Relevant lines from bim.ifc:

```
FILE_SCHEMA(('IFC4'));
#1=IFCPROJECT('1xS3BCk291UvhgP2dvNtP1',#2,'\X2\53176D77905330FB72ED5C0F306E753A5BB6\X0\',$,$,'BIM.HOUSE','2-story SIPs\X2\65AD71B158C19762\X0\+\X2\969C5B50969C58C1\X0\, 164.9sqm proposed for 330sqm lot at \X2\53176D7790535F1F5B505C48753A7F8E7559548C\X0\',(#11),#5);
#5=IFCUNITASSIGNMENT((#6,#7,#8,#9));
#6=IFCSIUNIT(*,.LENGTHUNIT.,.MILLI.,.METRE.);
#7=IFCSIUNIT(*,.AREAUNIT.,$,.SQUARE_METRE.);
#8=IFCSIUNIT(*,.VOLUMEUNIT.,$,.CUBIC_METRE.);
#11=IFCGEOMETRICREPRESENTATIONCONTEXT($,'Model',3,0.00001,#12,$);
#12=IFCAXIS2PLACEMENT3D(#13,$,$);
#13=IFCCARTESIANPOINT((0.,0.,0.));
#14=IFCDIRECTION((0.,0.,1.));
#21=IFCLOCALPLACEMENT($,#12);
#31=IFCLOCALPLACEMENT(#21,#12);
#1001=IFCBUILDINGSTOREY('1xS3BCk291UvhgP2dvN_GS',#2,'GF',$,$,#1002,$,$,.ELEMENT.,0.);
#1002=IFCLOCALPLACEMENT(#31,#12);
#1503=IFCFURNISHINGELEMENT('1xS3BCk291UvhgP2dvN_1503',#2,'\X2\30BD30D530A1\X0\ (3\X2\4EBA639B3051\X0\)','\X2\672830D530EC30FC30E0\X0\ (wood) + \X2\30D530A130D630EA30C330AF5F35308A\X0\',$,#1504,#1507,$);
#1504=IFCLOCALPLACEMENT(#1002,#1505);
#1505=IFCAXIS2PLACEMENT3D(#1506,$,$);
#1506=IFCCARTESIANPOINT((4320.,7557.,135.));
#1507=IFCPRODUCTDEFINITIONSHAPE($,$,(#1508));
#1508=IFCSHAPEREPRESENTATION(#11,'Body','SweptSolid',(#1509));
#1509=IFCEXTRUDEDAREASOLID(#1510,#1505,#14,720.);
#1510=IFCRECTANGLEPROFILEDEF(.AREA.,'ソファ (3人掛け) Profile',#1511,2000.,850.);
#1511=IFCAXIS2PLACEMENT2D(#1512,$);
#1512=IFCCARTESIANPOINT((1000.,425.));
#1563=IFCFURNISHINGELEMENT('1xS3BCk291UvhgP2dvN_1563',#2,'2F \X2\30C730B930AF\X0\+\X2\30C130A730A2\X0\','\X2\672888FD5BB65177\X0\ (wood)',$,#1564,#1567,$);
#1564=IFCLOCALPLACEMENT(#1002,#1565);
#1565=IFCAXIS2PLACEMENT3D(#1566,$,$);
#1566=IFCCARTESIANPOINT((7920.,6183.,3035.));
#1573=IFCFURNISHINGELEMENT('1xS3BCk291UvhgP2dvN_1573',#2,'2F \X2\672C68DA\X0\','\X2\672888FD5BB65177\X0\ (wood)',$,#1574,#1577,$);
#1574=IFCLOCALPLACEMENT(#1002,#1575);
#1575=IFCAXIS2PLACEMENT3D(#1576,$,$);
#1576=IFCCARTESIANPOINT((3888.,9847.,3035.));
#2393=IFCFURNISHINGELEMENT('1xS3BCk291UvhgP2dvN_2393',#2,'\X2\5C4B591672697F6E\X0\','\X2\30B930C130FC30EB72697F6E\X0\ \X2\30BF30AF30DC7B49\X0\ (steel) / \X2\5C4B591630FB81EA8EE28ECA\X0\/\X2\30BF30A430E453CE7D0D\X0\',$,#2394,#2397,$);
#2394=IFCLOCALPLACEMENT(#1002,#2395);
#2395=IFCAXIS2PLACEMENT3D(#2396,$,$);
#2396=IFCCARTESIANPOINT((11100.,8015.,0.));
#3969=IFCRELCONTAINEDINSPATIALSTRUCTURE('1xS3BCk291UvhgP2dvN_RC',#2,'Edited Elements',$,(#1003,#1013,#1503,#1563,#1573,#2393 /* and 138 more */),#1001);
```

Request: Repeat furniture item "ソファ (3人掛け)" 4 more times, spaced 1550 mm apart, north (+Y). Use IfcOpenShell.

```python
import numpy as np
import ifcopenshell
import ifcopenshell.api.geometry
import ifcopenshell.api.root
import ifcopenshell.util.element
import ifcopenshell.util.placement

model = ifcopenshell.open("bim.ifc")


def reuse_history(source, copy):
    """copy_class also copies each property set's owner history, people and application; keep the originals."""
    for rel in copy.IsDefinedBy:
        if rel.is_a("IfcRelDefinesByProperties") and (history := rel.RelatingPropertyDefinition.OwnerHistory):
            rel.RelatingPropertyDefinition.OwnerHistory = source.OwnerHistory
            ifcopenshell.util.element.remove_deep2(model, history)


source = model.by_guid("1xS3BCk291UvhgP2dvN_1503")
base = ifcopenshell.util.placement.get_local_placement(source.ObjectPlacement)
step = np.array([0.0, 1.0, 0.0]) * 1550.0

for i in range(1, 5):
    copy = ifcopenshell.api.root.copy_class(model, product=source)
    copy.Representation = ifcopenshell.util.element.copy_deep(
        model, source.Representation, exclude=["IfcGeometricRepresentationContext", "IfcRepresentationMap"]
    )
    reuse_history(source, copy)
    matrix = base.copy()
    matrix[:3, 3] += i * step
    print("added at", matrix[:3, 3].round(3) + 0.0)
    ifcopenshell.api.geometry.edit_object_placement(model, product=copy, matrix=matrix, is_si=False)

model.write("bim-out.ifc")
```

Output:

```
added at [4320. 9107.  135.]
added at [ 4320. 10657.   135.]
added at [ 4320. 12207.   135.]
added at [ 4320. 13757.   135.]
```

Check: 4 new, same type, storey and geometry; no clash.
